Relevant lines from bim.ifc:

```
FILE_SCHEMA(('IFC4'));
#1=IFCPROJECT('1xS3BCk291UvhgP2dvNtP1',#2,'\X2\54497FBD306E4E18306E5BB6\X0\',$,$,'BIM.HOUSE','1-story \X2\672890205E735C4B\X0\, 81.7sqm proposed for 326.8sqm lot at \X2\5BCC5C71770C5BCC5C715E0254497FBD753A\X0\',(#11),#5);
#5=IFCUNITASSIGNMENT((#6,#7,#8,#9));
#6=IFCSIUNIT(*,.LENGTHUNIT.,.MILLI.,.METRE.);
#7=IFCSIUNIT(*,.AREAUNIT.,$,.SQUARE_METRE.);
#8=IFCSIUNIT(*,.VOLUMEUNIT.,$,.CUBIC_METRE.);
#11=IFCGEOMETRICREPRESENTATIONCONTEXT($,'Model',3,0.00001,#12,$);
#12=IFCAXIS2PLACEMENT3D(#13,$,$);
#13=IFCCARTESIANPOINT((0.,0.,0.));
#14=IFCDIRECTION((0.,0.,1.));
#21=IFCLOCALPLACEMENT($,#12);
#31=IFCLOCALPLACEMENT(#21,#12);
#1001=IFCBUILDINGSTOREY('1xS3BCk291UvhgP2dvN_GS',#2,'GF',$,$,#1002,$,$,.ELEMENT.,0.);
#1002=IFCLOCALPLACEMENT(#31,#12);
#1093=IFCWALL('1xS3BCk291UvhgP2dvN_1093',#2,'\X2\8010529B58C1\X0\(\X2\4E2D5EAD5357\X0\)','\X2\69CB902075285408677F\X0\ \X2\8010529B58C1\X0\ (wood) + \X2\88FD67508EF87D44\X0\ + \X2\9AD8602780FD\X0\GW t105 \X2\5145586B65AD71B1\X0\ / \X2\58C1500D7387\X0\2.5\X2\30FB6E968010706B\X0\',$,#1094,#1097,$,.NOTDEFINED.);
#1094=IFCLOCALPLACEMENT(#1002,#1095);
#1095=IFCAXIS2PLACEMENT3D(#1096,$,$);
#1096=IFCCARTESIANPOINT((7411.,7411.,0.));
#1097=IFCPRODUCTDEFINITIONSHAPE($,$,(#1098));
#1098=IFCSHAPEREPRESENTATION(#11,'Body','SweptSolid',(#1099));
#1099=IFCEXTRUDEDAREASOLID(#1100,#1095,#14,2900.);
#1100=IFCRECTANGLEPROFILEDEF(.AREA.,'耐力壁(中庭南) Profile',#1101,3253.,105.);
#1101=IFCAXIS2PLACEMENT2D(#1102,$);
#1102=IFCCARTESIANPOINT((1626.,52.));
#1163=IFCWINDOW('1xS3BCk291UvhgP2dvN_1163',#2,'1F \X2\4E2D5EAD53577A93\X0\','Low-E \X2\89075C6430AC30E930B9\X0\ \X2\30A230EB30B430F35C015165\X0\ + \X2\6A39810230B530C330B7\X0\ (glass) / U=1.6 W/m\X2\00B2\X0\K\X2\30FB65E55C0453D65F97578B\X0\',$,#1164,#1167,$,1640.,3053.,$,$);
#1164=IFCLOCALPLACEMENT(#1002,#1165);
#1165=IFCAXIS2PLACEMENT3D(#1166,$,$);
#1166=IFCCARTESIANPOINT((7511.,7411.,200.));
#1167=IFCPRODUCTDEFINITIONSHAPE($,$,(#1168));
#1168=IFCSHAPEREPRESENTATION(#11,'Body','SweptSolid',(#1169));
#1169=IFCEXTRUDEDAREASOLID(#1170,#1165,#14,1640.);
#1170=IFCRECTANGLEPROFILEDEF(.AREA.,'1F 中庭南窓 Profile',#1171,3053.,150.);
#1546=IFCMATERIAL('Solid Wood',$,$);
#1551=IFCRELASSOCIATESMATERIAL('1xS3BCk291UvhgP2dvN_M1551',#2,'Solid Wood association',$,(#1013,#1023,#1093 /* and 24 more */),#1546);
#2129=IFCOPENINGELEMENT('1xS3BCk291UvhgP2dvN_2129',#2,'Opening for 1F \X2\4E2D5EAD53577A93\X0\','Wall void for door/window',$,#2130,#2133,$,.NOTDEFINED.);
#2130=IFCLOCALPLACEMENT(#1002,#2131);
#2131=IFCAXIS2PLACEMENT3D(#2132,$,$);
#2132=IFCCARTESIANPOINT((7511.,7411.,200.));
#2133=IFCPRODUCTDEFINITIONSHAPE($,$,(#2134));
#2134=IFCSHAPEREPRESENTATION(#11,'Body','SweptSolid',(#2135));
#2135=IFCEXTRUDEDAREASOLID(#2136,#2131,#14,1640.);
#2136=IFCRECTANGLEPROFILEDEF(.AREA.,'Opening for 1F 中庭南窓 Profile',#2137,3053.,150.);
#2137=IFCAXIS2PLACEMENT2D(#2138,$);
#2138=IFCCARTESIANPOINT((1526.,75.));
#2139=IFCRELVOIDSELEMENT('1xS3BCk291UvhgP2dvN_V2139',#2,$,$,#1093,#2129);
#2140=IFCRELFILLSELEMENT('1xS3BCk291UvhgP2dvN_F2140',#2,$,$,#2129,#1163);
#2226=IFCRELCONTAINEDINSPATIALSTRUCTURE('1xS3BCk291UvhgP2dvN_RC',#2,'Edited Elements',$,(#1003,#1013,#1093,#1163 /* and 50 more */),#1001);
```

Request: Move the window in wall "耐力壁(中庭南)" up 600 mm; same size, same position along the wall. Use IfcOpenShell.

```python
import numpy as np
import ifcopenshell
import ifcopenshell.api.geometry
import ifcopenshell.util.placement
import ifcopenshell.util.unit

model = ifcopenshell.open("bim.ifc")
unit_scale = ifcopenshell.util.unit.calculate_unit_scale(model)

window = model.by_id(1163)
opening = window.FillsVoids[0].RelatingOpeningElement
dz = 600.0

shift = np.array([0.0, 0.0, dz])
# The window is not placed relative to its opening, so move both.
for product in (opening, window):
    matrix = ifcopenshell.util.placement.get_local_placement(product.ObjectPlacement)
    matrix[:3, 3] += shift
    ifcopenshell.api.geometry.edit_object_placement(model, product=product, matrix=matrix, is_si=False)

print(f"moved by {dz * unit_scale:+.3f} m")

model.write("bim_v2.ifc")
```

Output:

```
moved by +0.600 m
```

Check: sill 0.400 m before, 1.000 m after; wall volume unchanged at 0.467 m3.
